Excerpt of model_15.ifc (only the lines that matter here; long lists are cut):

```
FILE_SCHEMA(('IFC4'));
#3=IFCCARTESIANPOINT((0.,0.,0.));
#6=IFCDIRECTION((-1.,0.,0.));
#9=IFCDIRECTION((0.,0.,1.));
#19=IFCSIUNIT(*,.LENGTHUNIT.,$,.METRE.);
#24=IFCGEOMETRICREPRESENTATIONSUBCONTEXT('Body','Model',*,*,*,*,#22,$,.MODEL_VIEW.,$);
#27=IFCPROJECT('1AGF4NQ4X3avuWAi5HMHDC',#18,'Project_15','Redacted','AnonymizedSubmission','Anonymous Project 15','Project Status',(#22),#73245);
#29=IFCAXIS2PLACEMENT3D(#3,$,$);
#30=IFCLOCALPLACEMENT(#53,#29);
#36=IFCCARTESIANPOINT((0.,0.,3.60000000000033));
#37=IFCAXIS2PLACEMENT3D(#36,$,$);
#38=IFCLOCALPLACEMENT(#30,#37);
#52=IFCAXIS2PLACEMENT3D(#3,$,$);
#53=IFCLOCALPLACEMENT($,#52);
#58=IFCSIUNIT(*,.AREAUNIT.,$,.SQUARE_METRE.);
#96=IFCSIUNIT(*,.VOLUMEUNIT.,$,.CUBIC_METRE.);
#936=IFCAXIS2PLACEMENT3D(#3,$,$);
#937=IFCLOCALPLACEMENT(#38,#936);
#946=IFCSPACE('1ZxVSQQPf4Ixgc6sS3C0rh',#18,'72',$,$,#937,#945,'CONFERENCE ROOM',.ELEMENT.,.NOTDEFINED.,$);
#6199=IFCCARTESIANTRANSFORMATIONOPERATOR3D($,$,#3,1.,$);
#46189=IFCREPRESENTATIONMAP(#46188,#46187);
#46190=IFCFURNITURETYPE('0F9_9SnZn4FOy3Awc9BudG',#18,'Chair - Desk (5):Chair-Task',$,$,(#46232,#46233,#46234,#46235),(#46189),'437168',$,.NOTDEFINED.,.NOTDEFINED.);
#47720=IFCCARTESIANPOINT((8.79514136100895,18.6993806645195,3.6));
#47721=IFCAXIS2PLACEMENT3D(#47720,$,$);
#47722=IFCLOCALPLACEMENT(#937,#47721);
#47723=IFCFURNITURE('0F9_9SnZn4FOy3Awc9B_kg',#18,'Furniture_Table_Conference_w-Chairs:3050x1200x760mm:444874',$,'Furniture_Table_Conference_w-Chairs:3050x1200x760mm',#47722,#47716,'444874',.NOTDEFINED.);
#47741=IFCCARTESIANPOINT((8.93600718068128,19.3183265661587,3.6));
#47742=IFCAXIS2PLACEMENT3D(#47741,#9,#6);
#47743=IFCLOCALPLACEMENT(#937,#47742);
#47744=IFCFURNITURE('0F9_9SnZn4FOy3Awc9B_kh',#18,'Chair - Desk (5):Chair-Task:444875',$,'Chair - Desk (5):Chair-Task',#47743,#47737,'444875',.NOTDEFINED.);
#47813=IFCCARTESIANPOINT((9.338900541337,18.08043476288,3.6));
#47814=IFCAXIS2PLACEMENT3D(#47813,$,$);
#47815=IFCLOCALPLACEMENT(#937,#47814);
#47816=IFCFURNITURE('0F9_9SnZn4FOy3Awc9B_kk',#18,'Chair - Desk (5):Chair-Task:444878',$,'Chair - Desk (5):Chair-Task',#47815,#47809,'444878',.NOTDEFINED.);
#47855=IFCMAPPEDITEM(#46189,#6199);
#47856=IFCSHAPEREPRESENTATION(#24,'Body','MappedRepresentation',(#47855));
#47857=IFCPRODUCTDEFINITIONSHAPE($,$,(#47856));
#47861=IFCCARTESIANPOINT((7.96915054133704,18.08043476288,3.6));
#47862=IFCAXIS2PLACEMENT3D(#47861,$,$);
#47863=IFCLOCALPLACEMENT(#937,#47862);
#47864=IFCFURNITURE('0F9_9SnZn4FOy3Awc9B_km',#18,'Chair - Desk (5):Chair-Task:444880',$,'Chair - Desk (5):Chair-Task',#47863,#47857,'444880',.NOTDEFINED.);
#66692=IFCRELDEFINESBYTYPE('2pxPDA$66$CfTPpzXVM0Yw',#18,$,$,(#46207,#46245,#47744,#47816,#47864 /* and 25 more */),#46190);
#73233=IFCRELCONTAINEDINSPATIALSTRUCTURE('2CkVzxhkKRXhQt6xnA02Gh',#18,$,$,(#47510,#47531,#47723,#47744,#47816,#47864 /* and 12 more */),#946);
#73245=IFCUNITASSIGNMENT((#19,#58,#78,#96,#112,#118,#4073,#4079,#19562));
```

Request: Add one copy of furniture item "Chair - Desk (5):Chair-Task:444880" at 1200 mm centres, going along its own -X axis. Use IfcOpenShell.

```python
import ifcopenshell
import ifcopenshell.api.geometry
import ifcopenshell.api.root
import ifcopenshell.util.element
import ifcopenshell.util.placement
import ifcopenshell.util.unit

model = ifcopenshell.open("model_15.ifc")
unit_scale = ifcopenshell.util.unit.calculate_unit_scale(model)


def reuse_history(source, copy):
    """copy_class also copies each property set's owner history, people and application; keep the originals."""
    for rel in copy.IsDefinedBy:
        if rel.is_a("IfcRelDefinesByProperties") and (history := rel.RelatingPropertyDefinition.OwnerHistory):
            rel.RelatingPropertyDefinition.OwnerHistory = source.OwnerHistory
            ifcopenshell.util.element.remove_deep2(model, history)


source = model.by_guid("0F9_9SnZn4FOy3Awc9B_km")
base = ifcopenshell.util.placement.get_local_placement(source.ObjectPlacement)
step = -base[:3, 0] * 1.2 / unit_scale

for i in range(1, 2):
    copy = ifcopenshell.api.root.copy_class(model, product=source)
    copy.Representation = ifcopenshell.util.element.copy_deep(
        model, source.Representation, exclude=["IfcGeometricRepresentationContext", "IfcRepresentationMap"]
    )
    copy.Name = "Chair - Desk (5):Chair-Task"
    copy.Tag = None
    reuse_history(source, copy)
    matrix = base.copy()
    matrix[:3, 3] += i * step
    print("added at", matrix[:3, 3].round(3) + 0.0)
    ifcopenshell.api.geometry.edit_object_placement(model, product=copy, matrix=matrix, is_si=False)

model.write("model_15_updated.ifc")
```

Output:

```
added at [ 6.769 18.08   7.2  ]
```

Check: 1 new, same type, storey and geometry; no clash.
